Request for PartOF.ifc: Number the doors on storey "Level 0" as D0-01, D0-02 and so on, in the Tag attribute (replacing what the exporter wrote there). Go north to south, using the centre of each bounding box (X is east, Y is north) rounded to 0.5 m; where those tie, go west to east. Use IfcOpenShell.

First a look at what the model holds.

```python
import ifcopenshell
import ifcopenshell.util.element
import ifcopenshell.util.placement

model = ifcopenshell.open("PartOF.ifc")
print(model.schema)
storey = next(s for s in model.by_type("IfcBuildingStorey") if s.Name == "Level 0")
doors = [e for e in ifcopenshell.util.element.get_decomposition(storey) if e.is_a("IfcDoor")]
for e in sorted(doors, key=lambda e: e.id()):
    origin = ifcopenshell.util.placement.get_local_placement(e.ObjectPlacement)[:3, 3]
    print(e.id(), e.Tag, e.Name, origin.round(2) + 0.0, sep=" | ")
```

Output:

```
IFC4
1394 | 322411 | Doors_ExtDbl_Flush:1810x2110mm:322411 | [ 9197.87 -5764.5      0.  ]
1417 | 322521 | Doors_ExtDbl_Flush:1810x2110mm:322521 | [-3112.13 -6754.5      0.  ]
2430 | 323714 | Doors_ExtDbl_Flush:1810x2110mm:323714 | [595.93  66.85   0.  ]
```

```python
import ifcopenshell
import ifcopenshell.geom
import ifcopenshell.util.element
import ifcopenshell.util.shape

model = ifcopenshell.open("PartOF.ifc")
settings = ifcopenshell.geom.settings()
settings.set("use-world-coords", True)


def centre(element):
    shape = ifcopenshell.geom.create_shape(settings, element)
    return ifcopenshell.util.shape.get_bbox_centroid(shape.geometry)


storey = next(s for s in model.by_type("IfcBuildingStorey") if s.Name == "Level 0")
doors = [e for e in ifcopenshell.util.element.get_decomposition(storey) if e.is_a("IfcDoor")]

# Insertion points can sit at a corner or the storey origin, so sort by the geometry (in metres).
centres = {e: centre(e) for e in doors}
doors.sort(key=lambda e: (-round(centres[e][1] / 0.5), centres[e][0]))

for i, e in enumerate(doors, start=1):
    number = f"D0-{i:02d}"
    e.Tag = number
    print(e.id(), number)

model.write("PartOF_v2.ifc")
```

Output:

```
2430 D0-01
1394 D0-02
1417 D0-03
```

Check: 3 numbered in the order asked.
